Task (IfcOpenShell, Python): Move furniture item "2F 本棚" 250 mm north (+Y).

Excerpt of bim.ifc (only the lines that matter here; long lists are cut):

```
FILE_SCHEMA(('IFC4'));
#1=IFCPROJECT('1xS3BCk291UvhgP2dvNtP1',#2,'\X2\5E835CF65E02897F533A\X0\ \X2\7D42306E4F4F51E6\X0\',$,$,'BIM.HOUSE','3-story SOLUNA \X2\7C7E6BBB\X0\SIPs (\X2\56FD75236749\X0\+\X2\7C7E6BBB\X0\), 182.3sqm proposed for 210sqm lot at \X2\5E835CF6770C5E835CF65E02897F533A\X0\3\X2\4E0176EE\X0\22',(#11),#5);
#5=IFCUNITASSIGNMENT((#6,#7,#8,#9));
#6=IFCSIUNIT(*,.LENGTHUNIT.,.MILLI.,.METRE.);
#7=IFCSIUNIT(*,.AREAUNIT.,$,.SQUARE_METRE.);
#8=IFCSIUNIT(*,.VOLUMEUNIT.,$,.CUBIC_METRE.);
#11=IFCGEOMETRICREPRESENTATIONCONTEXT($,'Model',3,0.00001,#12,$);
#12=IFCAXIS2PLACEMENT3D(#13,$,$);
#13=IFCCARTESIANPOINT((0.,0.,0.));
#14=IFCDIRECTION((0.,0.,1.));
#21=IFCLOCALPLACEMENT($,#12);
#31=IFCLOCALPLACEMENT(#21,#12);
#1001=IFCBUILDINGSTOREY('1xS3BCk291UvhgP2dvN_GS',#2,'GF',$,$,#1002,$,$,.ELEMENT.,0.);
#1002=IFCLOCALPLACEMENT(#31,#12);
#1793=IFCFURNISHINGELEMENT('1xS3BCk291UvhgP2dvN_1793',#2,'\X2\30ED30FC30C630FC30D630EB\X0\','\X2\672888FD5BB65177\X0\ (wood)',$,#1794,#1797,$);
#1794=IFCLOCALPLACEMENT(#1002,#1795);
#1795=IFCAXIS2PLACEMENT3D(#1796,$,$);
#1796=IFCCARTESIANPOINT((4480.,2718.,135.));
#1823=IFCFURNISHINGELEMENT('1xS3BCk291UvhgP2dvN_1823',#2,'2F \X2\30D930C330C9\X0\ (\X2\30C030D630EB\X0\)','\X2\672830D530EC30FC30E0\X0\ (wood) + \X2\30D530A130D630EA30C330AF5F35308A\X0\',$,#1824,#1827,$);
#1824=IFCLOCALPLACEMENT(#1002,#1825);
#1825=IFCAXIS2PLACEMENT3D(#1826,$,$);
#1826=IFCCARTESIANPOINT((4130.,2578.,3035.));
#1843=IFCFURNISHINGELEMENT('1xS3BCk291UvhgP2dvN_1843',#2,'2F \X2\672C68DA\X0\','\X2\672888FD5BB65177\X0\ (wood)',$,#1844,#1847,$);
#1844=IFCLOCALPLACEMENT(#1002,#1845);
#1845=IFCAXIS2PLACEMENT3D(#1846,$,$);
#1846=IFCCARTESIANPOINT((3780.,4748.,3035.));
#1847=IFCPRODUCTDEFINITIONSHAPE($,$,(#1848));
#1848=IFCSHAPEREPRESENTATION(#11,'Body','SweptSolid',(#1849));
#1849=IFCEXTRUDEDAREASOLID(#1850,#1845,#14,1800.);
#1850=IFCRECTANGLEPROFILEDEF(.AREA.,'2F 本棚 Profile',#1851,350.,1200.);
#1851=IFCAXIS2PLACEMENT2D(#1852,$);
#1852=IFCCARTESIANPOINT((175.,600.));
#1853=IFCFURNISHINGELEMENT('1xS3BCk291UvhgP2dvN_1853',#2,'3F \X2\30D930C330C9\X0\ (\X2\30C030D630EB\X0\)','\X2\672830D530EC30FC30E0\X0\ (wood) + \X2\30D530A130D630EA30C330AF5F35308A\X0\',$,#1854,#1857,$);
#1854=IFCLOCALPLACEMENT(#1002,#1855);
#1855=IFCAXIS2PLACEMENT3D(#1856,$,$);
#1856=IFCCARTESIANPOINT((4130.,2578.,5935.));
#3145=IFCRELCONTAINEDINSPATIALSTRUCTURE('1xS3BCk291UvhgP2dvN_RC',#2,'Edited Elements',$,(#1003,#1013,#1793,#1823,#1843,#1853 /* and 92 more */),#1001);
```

```python
import ifcopenshell
import ifcopenshell.api.geometry
import ifcopenshell.util.placement
import ifcopenshell.util.unit

model = ifcopenshell.open("bim.ifc")
unit_scale = ifcopenshell.util.unit.calculate_unit_scale(model)

item = model.by_id(1843)
matrix = ifcopenshell.util.placement.get_local_placement(item.ObjectPlacement)
matrix[1, 3] += 0.25 / unit_scale
ifcopenshell.api.geometry.edit_object_placement(model, product=item, matrix=matrix, is_si=False)

print(ifcopenshell.util.placement.get_local_placement(item.ObjectPlacement).round(3) + 0.0)

model.write("bim-out.ifc")
```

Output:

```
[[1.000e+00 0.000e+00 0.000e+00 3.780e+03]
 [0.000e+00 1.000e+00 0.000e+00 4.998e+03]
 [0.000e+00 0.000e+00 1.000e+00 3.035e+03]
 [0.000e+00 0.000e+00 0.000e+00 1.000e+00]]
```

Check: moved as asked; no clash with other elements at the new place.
